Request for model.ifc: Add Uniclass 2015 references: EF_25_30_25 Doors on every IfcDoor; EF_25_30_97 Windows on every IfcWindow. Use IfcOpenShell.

First a look at what the model holds.

```python
import ifcopenshell

model = ifcopenshell.open("model.ifc")
print(model.schema)
print("classifications:", [c.Name for c in model.by_type("IfcClassification")])
for ifc_class in ("IfcDoor", "IfcRoof", "IfcStair", "IfcWall", "IfcWindow"):
    print(ifc_class, len(model.by_type(ifc_class)))
```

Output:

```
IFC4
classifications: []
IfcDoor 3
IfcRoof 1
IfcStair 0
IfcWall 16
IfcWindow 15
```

```python
import ifcopenshell
import ifcopenshell.api.classification

model = ifcopenshell.open("model.ifc")

system = ifcopenshell.api.classification.add_classification(model, classification="Uniclass 2015")

codes = {
    "IfcDoor": ("EF_25_30_25", "Doors"),
    "IfcWindow": ("EF_25_30_97", "Windows"),
}
for ifc_class, (code, name) in codes.items():
    products = model.by_type(ifc_class)
    ifcopenshell.api.classification.add_reference(
        model, products=products, classification=system, identification=code, name=name
    )
    print(code, len(products))

model.write("model_v2.ifc")
```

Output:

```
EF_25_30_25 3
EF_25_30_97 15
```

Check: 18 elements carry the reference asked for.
